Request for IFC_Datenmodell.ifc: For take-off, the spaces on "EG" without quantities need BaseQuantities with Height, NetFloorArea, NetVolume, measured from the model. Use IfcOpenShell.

First a look at what the model holds.

```python
import ifcopenshell
import ifcopenshell.util.element
import ifcopenshell.util.unit

model = ifcopenshell.open("IFC_Datenmodell.ifc")
print(model.schema)
for unit_type in ("LENGTHUNIT", "AREAUNIT", "VOLUMEUNIT"):
    print(unit_type, ifcopenshell.util.unit.calculate_unit_scale(model, unit_type))
storey = next(s for s in model.by_type("IfcBuildingStorey") if s.Name == "EG")
spaces = [e for e in ifcopenshell.util.element.get_decomposition(storey) if e.is_a("IfcSpace")]
for e in sorted(spaces, key=lambda e: e.id()):
    print(e.id(), e.is_a(), e.Name, list(ifcopenshell.util.element.get_psets(e, qtos_only=True)), sep=" | ")
```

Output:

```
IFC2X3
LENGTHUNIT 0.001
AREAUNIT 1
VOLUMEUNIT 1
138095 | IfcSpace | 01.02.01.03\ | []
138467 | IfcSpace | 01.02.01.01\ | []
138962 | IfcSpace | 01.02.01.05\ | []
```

```python
import ifcopenshell
import ifcopenshell.api.pset
import ifcopenshell.geom
import ifcopenshell.util.element
import ifcopenshell.util.shape
import ifcopenshell.util.unit

model = ifcopenshell.open("IFC_Datenmodell.ifc")
unit_scale = ifcopenshell.util.unit.calculate_unit_scale(model)
area_scale = ifcopenshell.util.unit.calculate_unit_scale(model, "AREAUNIT")
volume_scale = ifcopenshell.util.unit.calculate_unit_scale(model, "VOLUMEUNIT")
settings = ifcopenshell.geom.settings()

storey = next(s for s in model.by_type("IfcBuildingStorey") if s.Name == "EG")
spaces = [e for e in ifcopenshell.util.element.get_decomposition(storey) if e.is_a("IfcSpace")]

for e in sorted(spaces, key=lambda e: e.id()):
    if ifcopenshell.util.element.get_psets(e, qtos_only=True, should_inherit=False):
        continue
    # Geometry comes back in metres, in the element's own axes.
    shape = ifcopenshell.geom.create_shape(settings, e)
    values = {
        "Height": ifcopenshell.util.shape.get_z(shape.geometry) / unit_scale,
        "NetFloorArea": ifcopenshell.util.shape.get_footprint_area(shape.geometry) / area_scale,
        "NetVolume": ifcopenshell.util.shape.get_volume(shape.geometry) / volume_scale,
    }
    qto = ifcopenshell.api.pset.add_qto(model, product=e, name="BaseQuantities")
    ifcopenshell.api.pset.edit_qto(model, qto=qto, properties=values)
    print(e.id(), {k: round(v, 3) for k, v in values.items()})

model.write("IFC_Datenmodell-out.ifc")
```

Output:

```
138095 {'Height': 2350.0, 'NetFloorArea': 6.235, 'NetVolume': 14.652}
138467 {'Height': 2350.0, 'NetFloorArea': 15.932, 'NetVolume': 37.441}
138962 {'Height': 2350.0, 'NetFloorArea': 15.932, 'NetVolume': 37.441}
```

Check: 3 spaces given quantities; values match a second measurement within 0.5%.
